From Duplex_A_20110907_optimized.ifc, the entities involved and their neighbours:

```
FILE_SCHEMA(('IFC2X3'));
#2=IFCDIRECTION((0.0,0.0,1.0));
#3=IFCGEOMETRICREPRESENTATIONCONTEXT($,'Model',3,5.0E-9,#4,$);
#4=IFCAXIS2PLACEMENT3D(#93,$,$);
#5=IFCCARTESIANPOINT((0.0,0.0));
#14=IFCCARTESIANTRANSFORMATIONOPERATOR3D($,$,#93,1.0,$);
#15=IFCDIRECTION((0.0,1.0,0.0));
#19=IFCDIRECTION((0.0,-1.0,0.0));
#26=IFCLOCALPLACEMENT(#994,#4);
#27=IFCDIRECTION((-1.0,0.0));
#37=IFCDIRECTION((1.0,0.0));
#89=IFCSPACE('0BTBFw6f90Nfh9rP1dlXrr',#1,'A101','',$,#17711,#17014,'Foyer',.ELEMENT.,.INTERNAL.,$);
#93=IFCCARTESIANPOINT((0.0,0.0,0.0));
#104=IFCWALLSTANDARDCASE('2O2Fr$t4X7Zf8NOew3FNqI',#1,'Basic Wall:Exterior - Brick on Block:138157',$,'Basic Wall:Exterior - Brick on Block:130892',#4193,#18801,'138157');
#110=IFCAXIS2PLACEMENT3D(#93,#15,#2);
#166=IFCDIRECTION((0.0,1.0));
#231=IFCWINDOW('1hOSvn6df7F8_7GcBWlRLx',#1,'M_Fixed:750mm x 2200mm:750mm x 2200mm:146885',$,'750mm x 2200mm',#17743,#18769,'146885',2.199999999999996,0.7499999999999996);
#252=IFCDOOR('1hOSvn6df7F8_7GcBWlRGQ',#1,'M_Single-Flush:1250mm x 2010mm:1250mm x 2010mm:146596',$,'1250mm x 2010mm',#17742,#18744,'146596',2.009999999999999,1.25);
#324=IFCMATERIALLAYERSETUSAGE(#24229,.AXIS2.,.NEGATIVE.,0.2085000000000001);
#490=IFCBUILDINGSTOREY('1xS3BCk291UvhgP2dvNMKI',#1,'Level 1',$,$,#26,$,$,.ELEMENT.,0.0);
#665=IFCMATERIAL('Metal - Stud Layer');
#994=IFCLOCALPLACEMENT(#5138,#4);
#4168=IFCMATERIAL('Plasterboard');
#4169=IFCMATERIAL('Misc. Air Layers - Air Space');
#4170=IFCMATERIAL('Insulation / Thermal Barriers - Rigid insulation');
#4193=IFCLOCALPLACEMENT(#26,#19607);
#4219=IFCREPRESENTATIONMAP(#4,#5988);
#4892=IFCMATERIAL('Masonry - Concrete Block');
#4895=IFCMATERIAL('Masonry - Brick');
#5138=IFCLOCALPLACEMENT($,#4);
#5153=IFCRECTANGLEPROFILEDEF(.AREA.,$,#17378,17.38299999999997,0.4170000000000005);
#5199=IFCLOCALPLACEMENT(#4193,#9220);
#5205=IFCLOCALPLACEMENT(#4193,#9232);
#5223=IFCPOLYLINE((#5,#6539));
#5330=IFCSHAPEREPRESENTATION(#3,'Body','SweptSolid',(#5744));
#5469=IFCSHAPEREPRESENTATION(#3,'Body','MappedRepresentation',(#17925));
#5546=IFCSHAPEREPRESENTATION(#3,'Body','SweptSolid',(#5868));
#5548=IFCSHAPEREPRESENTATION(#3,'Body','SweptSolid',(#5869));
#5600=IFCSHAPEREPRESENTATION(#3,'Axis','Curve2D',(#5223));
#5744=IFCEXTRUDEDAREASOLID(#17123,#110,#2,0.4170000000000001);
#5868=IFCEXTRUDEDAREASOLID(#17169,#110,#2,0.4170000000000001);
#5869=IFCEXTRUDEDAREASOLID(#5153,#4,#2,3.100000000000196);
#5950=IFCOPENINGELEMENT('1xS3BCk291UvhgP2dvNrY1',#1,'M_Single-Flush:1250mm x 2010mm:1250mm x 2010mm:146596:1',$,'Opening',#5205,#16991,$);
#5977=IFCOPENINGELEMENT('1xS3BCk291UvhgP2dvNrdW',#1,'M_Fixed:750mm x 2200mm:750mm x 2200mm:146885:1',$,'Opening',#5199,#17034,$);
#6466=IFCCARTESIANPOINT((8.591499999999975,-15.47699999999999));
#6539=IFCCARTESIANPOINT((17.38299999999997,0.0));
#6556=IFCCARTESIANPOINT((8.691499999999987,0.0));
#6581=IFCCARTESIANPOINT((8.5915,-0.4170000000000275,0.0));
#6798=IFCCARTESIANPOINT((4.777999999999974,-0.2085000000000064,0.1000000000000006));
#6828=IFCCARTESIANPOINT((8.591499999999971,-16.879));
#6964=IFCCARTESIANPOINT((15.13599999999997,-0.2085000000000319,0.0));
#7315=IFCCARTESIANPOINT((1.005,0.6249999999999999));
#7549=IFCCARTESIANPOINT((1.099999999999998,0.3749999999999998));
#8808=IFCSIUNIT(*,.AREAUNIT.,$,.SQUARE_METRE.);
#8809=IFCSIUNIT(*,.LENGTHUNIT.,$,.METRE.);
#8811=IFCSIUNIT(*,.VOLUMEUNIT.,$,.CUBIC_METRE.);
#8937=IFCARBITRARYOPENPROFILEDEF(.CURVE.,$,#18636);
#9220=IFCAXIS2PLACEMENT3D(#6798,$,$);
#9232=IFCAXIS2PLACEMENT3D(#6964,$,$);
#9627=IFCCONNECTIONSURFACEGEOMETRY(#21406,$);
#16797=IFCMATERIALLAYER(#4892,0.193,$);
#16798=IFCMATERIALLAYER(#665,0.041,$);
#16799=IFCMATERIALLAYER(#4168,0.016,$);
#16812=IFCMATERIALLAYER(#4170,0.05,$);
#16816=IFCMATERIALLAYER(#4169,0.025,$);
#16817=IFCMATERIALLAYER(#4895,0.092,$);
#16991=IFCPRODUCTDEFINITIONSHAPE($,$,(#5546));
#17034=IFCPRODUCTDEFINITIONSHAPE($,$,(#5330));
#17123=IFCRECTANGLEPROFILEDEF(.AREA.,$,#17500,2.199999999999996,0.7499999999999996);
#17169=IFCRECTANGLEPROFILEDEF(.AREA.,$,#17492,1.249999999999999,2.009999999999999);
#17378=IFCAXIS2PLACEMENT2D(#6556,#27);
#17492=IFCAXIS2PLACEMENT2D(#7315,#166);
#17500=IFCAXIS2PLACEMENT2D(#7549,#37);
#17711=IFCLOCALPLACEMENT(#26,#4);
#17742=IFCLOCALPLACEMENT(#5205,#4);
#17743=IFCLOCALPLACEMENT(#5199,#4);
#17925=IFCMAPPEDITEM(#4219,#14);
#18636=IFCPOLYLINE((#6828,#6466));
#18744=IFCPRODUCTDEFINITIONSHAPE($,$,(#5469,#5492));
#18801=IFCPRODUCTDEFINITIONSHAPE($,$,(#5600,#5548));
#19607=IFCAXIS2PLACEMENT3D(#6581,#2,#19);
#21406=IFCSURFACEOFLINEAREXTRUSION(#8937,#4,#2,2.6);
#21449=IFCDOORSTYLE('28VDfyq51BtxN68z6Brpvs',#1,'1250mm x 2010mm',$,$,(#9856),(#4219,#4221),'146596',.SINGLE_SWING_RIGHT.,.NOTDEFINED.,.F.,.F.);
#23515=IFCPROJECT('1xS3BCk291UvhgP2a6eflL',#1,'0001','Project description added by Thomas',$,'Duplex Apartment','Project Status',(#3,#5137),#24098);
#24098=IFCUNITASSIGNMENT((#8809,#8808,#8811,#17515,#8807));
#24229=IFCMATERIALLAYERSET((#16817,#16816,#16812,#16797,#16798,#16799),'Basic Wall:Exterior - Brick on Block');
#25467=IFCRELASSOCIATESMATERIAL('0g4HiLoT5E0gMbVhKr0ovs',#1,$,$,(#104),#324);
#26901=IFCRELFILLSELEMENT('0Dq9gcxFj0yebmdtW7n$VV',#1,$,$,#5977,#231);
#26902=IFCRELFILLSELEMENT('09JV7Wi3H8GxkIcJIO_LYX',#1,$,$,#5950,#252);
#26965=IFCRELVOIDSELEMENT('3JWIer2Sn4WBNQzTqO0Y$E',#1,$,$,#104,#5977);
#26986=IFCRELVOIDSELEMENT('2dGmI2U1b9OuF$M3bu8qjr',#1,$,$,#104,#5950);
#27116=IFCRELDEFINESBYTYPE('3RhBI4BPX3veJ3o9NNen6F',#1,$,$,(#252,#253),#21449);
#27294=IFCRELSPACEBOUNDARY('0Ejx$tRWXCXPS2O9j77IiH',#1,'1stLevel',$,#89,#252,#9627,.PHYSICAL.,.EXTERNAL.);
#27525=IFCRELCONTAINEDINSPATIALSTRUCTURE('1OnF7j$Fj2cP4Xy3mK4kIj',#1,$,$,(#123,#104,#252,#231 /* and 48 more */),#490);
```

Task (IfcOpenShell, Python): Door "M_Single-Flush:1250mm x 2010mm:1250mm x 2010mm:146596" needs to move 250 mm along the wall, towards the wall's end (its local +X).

```python
import numpy as np
import ifcopenshell
import ifcopenshell.api.geometry
import ifcopenshell.util.placement

model = ifcopenshell.open("Duplex_A_20110907_optimized.ifc")

door = model.by_guid("1hOSvn6df7F8_7GcBWlRGQ")
opening = door.FillsVoids[0].RelatingOpeningElement
wall = opening.VoidsElements[0].RelatingBuildingElement

wall_matrix = ifcopenshell.util.placement.get_local_placement(wall.ObjectPlacement)
shift = wall_matrix[:3, 0] * 0.25
before = ifcopenshell.util.placement.get_local_placement(door.ObjectPlacement)[:3, 3].copy()

# The door is placed relative to its opening, so it follows when the opening moves.
matrix = ifcopenshell.util.placement.get_local_placement(opening.ObjectPlacement)
matrix[:3, 3] += shift
ifcopenshell.api.geometry.edit_object_placement(
    model, product=opening, matrix=matrix, is_si=False, should_transform_children=True
)

# Space boundary surfaces are stored in each space's coordinates; move them too.
for rel in door.ProvidesBoundaries:
    if not rel.ConnectionGeometry:
        continue
    surface = rel.ConnectionGeometry.SurfaceOnRelatingElement
    space_matrix = ifcopenshell.util.placement.get_local_placement(rel.RelatingSpace.ObjectPlacement)
    point = np.array(surface.Position.Location.Coordinates) + space_matrix[:3, :3].T @ shift
    surface.Position = model.createIfcAxis2Placement3D(
        model.createIfcCartesianPoint(point.tolist()), surface.Position.Axis, surface.Position.RefDirection
    )

after = ifcopenshell.util.placement.get_local_placement(door.ObjectPlacement)[:3, 3]
print("door moved by", (after - before).round(3) + 0.0)

model.write("Duplex_A_20110907_optimized_rev.ifc")
```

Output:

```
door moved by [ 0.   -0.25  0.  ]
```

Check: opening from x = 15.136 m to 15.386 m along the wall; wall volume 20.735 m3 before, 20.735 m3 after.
